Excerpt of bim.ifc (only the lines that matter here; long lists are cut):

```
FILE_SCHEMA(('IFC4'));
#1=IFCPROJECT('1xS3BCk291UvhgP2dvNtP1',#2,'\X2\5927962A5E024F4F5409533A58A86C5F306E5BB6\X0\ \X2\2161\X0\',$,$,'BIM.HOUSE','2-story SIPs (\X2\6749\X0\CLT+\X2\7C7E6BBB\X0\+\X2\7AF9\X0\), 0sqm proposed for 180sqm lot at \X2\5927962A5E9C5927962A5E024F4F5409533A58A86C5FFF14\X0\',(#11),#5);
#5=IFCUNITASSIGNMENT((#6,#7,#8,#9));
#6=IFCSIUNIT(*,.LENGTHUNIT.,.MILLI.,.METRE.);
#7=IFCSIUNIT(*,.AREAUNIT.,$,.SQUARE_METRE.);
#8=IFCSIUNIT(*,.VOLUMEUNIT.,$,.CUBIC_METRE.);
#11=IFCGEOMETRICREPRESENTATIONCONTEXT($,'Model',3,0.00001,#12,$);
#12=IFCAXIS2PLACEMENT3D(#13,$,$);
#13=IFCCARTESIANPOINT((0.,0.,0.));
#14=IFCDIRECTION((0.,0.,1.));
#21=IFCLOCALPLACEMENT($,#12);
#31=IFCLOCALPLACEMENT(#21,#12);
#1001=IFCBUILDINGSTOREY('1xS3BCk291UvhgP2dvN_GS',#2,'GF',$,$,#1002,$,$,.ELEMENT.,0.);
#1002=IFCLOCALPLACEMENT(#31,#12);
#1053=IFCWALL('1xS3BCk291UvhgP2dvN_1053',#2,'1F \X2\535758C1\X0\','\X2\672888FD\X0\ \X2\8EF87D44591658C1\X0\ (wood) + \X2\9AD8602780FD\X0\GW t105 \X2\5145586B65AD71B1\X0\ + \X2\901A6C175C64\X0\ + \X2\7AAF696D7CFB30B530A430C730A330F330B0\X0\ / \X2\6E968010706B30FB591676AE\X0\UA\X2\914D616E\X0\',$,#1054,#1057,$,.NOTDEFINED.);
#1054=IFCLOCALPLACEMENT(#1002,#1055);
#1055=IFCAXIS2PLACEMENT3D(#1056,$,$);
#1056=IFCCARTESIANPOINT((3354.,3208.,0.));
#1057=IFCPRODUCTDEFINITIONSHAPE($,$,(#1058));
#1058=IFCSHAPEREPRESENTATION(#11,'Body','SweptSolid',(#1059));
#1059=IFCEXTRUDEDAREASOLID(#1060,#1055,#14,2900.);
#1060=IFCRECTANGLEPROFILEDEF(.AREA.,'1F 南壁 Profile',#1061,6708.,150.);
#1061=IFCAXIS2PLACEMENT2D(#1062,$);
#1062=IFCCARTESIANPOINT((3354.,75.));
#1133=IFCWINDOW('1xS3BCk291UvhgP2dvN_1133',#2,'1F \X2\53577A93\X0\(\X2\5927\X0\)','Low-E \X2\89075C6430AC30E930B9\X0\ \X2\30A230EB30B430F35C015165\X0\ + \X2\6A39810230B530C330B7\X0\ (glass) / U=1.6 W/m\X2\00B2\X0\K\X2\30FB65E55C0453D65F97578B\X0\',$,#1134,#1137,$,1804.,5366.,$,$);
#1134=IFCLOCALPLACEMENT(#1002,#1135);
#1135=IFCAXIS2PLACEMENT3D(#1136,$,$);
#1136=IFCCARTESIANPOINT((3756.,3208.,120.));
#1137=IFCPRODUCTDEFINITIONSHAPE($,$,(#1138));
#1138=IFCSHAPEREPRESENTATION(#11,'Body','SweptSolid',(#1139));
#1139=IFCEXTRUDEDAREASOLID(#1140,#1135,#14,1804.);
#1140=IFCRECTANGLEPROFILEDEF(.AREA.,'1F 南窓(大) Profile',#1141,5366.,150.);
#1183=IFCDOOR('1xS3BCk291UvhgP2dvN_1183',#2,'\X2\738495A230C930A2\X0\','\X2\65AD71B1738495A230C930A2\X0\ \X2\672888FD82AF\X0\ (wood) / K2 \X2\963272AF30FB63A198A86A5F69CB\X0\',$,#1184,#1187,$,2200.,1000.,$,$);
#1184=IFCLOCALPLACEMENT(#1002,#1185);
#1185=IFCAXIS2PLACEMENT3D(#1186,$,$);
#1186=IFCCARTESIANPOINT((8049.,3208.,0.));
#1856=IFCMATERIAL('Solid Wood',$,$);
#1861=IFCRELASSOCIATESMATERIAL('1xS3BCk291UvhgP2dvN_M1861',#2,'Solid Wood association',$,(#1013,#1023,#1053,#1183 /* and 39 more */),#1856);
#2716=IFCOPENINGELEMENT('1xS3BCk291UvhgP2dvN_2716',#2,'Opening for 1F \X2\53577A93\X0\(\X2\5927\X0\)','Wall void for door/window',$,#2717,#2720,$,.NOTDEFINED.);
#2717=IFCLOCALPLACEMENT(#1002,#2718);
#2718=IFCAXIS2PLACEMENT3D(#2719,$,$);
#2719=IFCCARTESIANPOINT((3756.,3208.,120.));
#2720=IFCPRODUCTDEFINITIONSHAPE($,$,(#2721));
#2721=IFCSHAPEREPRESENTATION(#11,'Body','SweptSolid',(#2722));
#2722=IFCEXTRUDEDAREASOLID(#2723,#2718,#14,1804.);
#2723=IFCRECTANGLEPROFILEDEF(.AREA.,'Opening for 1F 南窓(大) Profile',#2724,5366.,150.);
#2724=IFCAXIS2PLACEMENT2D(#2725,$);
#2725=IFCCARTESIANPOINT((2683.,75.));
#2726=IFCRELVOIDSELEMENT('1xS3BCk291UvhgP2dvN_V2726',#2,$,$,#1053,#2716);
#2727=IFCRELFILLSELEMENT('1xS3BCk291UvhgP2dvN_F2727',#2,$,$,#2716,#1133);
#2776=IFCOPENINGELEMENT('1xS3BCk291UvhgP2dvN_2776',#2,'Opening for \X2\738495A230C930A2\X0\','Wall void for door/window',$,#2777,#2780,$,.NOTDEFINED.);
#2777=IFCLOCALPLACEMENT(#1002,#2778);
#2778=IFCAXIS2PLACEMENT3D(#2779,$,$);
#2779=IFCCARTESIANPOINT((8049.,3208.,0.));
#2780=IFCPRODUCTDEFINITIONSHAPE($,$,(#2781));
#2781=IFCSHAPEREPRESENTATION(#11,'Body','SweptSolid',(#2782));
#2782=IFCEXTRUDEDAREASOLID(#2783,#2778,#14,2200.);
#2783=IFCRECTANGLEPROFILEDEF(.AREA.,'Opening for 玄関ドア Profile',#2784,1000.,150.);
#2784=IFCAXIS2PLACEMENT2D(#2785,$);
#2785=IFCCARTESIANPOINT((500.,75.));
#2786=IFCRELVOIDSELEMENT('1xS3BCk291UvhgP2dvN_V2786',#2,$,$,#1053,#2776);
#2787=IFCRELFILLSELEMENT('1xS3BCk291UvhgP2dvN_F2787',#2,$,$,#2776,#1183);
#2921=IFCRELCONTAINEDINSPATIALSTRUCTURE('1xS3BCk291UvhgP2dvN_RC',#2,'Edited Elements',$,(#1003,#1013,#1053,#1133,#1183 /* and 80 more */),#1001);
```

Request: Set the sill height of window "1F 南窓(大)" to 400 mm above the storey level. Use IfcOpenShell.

```python
import numpy as np
import ifcopenshell
import ifcopenshell.api.geometry
import ifcopenshell.geom
import ifcopenshell.util.element
import ifcopenshell.util.placement
import ifcopenshell.util.shape
import ifcopenshell.util.unit

model = ifcopenshell.open("bim.ifc")
unit_scale = ifcopenshell.util.unit.calculate_unit_scale(model)

window = model.by_id(1133)
opening = window.FillsVoids[0].RelatingOpeningElement
storey = ifcopenshell.util.element.get_container(window, ifc_class="IfcBuildingStorey")
level = ifcopenshell.util.placement.get_local_placement(storey.ObjectPlacement)[2, 3]

# The opening's origin need not be at the sill, so measure its lowest point.
shape = ifcopenshell.geom.create_shape(ifcopenshell.geom.settings(), opening)
bottom = ifcopenshell.util.shape.get_shape_bottom_elevation(shape, shape.geometry) / unit_scale
dz = level + 400.0 - bottom

shift = np.array([0.0, 0.0, dz])
# The window is not placed relative to its opening, so move both.
for product in (opening, window):
    matrix = ifcopenshell.util.placement.get_local_placement(product.ObjectPlacement)
    matrix[:3, 3] += shift
    ifcopenshell.api.geometry.edit_object_placement(model, product=product, matrix=matrix, is_si=False)

print(f"moved by {dz * unit_scale:+.3f} m")

model.write("bim_edited.ifc")
```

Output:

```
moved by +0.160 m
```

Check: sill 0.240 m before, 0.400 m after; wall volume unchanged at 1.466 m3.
